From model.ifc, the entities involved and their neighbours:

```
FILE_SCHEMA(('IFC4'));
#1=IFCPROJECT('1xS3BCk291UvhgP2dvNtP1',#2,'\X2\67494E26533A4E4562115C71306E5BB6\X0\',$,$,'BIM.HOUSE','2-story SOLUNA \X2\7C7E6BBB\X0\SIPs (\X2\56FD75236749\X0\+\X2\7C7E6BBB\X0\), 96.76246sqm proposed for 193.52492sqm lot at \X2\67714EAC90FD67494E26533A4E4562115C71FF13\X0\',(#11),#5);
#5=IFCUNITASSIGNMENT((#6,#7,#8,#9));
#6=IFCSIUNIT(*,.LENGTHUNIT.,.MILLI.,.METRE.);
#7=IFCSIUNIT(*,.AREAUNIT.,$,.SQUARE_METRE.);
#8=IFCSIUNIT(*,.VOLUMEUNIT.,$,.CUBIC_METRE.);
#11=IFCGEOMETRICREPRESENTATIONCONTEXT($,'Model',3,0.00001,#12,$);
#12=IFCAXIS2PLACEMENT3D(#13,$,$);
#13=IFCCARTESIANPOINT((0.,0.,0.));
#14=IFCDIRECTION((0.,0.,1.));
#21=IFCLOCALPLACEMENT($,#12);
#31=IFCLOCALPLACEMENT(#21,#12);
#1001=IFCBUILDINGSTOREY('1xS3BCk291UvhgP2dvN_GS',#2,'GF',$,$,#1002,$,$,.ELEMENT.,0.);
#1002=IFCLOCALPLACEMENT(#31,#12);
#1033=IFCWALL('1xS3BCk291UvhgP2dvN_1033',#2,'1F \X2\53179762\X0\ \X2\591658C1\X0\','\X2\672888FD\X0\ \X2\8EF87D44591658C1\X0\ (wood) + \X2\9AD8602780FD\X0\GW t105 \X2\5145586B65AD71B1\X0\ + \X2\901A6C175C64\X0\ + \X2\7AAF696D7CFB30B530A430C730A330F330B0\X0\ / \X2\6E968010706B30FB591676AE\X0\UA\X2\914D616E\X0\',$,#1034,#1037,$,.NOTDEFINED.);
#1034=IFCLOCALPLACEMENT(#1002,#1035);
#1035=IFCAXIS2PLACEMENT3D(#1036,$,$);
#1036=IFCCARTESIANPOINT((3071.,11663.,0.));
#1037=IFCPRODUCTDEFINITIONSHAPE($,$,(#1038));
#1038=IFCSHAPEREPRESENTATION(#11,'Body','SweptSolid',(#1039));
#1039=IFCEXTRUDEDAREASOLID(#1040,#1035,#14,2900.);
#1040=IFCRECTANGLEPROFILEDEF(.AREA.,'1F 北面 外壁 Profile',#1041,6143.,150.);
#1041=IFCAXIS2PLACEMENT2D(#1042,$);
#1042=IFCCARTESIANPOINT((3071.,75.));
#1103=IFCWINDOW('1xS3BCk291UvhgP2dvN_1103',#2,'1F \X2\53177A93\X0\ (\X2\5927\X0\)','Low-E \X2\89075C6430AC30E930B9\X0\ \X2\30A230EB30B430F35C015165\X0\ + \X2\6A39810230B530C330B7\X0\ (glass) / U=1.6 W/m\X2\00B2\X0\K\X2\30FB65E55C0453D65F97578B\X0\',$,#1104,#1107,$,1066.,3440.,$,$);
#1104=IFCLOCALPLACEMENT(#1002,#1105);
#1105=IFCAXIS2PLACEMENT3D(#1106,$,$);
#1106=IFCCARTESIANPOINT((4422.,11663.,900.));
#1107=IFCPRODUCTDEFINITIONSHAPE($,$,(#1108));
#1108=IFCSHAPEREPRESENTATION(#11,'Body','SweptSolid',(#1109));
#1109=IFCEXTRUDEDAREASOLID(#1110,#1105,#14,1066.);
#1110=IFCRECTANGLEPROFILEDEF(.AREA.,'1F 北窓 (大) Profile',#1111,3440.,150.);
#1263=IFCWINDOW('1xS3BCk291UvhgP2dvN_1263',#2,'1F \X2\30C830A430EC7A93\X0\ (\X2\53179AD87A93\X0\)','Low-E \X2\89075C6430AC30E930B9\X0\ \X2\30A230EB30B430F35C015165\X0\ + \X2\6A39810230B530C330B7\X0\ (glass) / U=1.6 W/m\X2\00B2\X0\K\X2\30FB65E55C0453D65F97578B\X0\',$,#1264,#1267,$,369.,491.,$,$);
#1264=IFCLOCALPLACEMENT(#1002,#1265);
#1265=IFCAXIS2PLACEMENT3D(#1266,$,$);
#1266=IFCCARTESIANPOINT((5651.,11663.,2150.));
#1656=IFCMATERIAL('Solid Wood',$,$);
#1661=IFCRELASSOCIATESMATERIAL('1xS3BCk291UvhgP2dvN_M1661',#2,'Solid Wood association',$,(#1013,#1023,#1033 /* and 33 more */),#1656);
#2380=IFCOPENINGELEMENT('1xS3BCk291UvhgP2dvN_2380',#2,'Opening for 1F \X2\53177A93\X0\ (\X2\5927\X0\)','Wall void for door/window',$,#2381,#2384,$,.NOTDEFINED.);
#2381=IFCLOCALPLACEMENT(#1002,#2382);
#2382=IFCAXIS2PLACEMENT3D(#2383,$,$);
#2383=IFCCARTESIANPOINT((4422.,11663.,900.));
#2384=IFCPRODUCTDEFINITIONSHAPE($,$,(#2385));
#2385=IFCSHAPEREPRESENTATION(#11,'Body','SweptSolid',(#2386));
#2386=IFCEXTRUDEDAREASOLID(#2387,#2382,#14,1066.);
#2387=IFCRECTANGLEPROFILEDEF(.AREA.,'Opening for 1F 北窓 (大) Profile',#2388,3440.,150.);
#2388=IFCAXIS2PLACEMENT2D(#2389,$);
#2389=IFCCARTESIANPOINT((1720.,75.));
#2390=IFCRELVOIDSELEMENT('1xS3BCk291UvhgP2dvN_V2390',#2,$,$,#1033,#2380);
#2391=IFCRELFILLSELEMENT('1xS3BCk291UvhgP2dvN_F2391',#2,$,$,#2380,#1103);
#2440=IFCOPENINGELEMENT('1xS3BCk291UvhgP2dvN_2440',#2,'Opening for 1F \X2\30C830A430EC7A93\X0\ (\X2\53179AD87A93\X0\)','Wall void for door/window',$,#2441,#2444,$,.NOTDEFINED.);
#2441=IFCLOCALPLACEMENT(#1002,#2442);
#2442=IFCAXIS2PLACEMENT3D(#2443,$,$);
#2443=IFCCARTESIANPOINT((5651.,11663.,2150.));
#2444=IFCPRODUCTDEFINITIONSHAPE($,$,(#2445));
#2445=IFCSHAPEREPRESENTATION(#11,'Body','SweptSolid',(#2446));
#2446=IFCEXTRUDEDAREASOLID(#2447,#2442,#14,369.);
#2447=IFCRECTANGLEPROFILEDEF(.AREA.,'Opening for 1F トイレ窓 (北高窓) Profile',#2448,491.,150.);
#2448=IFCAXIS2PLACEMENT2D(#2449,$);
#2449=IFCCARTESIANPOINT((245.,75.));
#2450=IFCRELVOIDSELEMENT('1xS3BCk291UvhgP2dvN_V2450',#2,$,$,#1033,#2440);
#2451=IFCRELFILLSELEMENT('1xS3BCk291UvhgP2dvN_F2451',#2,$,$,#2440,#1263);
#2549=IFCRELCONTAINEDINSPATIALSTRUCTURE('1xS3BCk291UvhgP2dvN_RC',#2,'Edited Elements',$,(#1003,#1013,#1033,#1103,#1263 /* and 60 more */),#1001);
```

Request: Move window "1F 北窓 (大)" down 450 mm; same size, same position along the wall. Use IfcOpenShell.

```python
import numpy as np
import ifcopenshell
import ifcopenshell.api.geometry
import ifcopenshell.util.placement
import ifcopenshell.util.unit

model = ifcopenshell.open("model.ifc")
unit_scale = ifcopenshell.util.unit.calculate_unit_scale(model)

window = model.by_guid("1xS3BCk291UvhgP2dvN_1103")
opening = window.FillsVoids[0].RelatingOpeningElement
dz = -450.0

shift = np.array([0.0, 0.0, dz])
# The window is not placed relative to its opening, so move both.
for product in (opening, window):
    matrix = ifcopenshell.util.placement.get_local_placement(product.ObjectPlacement)
    matrix[:3, 3] += shift
    ifcopenshell.api.geometry.edit_object_placement(model, product=product, matrix=matrix, is_si=False)

print(f"moved by {dz * unit_scale:+.3f} m")

model.write("model_v2.ifc")
```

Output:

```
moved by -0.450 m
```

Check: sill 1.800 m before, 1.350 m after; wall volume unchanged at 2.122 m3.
